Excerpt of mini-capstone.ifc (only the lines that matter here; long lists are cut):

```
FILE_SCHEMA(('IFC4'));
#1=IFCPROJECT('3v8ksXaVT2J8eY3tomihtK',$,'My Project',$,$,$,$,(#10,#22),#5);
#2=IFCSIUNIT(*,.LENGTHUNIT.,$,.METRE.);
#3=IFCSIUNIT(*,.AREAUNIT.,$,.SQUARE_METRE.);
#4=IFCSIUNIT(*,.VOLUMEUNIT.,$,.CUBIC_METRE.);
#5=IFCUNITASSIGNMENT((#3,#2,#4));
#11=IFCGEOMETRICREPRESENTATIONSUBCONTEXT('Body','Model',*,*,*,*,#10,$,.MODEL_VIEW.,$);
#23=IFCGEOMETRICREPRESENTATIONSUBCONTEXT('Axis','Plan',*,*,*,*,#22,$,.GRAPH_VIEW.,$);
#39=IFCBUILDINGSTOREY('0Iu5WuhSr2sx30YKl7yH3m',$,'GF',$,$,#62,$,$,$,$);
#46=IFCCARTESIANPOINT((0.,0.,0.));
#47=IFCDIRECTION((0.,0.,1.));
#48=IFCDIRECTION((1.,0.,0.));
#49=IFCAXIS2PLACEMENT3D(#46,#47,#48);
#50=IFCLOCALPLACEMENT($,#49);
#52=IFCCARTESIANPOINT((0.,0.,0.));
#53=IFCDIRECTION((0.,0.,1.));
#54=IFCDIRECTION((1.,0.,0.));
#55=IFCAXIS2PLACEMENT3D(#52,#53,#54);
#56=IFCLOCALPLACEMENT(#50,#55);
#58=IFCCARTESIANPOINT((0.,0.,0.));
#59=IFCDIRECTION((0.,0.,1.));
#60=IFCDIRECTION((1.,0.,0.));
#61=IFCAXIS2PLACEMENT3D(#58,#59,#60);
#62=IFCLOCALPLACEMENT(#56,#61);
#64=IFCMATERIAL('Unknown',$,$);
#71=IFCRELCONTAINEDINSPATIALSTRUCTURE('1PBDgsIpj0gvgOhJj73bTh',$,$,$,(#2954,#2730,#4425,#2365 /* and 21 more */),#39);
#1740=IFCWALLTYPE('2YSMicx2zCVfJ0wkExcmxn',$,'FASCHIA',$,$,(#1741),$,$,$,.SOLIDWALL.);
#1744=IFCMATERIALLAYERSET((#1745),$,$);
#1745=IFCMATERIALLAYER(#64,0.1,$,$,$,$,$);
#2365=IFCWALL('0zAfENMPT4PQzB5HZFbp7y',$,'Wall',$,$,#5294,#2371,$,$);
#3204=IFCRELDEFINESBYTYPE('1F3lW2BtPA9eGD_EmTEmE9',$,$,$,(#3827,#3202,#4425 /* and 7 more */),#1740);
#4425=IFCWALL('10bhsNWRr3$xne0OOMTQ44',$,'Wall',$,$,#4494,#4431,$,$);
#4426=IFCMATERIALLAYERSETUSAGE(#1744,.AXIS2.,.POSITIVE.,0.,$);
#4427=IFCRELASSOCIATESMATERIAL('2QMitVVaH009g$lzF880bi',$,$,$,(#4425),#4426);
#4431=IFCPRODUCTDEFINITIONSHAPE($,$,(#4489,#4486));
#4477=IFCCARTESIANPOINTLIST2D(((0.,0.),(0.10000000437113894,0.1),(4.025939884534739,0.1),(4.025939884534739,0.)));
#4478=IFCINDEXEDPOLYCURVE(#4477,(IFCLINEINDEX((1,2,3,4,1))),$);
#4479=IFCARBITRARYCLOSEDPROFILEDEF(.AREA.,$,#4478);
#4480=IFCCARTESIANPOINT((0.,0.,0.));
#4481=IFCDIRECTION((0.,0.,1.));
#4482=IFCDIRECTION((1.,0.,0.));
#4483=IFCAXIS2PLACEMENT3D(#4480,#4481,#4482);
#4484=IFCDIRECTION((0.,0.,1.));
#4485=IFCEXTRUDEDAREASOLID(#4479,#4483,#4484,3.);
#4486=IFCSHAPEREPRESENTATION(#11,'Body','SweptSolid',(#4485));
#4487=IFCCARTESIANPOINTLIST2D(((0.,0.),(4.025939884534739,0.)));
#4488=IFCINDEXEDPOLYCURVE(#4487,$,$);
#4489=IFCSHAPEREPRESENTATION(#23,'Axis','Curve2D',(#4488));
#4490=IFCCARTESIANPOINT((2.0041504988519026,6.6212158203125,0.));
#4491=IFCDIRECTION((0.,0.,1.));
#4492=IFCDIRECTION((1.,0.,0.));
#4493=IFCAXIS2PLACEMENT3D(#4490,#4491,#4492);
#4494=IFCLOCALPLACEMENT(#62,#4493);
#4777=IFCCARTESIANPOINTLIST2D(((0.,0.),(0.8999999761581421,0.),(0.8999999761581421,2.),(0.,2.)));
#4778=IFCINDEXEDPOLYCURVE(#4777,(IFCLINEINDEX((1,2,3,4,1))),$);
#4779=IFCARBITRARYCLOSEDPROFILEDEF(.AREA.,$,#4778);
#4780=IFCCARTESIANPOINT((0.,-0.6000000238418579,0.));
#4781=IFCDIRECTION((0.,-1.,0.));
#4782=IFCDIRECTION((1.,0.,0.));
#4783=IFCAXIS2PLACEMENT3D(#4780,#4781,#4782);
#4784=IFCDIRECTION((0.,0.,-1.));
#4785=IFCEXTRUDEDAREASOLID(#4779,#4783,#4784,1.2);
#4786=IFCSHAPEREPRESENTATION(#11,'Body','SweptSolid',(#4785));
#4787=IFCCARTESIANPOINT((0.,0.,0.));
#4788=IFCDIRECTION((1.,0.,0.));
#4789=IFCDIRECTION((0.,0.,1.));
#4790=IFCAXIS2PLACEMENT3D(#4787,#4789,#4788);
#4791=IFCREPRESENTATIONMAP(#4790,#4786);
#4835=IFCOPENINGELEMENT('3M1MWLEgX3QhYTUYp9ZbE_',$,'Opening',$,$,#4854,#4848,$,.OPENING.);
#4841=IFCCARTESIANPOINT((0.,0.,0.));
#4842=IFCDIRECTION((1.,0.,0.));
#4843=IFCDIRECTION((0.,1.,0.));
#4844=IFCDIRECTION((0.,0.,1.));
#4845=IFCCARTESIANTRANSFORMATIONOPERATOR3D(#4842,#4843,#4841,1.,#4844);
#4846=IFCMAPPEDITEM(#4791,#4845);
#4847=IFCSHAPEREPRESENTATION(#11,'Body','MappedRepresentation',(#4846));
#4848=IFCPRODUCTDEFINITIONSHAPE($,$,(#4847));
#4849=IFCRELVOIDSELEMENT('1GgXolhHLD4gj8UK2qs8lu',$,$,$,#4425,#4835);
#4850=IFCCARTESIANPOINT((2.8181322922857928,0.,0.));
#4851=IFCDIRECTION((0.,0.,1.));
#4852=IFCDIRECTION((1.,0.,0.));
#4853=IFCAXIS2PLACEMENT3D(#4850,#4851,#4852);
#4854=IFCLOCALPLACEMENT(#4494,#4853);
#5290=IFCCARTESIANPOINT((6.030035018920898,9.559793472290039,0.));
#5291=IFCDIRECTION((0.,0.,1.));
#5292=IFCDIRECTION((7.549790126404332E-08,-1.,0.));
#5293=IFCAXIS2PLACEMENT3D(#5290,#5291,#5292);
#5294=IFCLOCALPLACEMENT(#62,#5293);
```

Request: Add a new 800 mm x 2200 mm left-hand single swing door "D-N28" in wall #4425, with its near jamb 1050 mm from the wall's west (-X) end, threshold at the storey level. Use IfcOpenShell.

```python
import numpy as np
import ifcopenshell
import ifcopenshell.api.feature
import ifcopenshell.api.geometry
import ifcopenshell.api.root
import ifcopenshell.api.spatial
import ifcopenshell.geom
import ifcopenshell.util.element
import ifcopenshell.util.placement
import ifcopenshell.util.representation
import ifcopenshell.util.shape
import ifcopenshell.util.unit

model = ifcopenshell.open("mini-capstone.ifc")
unit_scale = ifcopenshell.util.unit.calculate_unit_scale(model)
settings = ifcopenshell.geom.settings()


def volume(element):
    """Net volume in cubic metres, openings subtracted."""
    shape = ifcopenshell.geom.create_shape(settings, element)
    return ifcopenshell.util.shape.get_volume(shape.geometry)


wall = model.by_id(4425)
storey = ifcopenshell.util.element.get_container(wall, ifc_class="IfcBuildingStorey")
context = ifcopenshell.util.representation.get_context(model, "Model", "Body", "MODEL_VIEW")
before = volume(wall)

width, height, from_end, sill = 0.8, 2.2, 1.05, 0.0  # metres

# The wall runs along its own X axis, and the end named is its -X end.
wall_shape = ifcopenshell.geom.create_shape(settings, wall)
x, y, z = ifcopenshell.util.shape.get_vertices(wall_shape.geometry).T
start = x.min() + from_end
face, thickness = float(y.min()), float(y.max() - y.min())
wall_matrix = ifcopenshell.util.placement.get_local_placement(wall.ObjectPlacement)
level = ifcopenshell.util.placement.get_local_placement(storey.ObjectPlacement)[2, 3]


def in_wall(x, y):
    """Placement at x, y metres in the wall's axes, at sill height."""
    matrix = wall_matrix.copy()
    matrix[:, 3] = wall_matrix @ np.array([x / unit_scale, y / unit_scale, 0.0, 1.0])
    matrix[2, 3] = level + sill / unit_scale
    return matrix


# Opening: a box that overshoots both wall faces by 50 mm.
opening = ifcopenshell.api.root.create_entity(model, ifc_class="IfcOpeningElement", predefined_type="OPENING")
box = ifcopenshell.api.geometry.add_wall_representation(
    model, context=context, length=width, height=height, thickness=thickness + 0.1
)
ifcopenshell.api.geometry.assign_representation(model, product=opening, representation=box)
ifcopenshell.api.geometry.edit_object_placement(model, product=opening, matrix=in_wall(start, face - 0.05), is_si=False)
ifcopenshell.api.feature.add_feature(model, feature=opening, element=wall)

door = ifcopenshell.api.root.create_entity(model, ifc_class="IfcDoor", name="D-N28", predefined_type="DOOR")
door.OverallWidth, door.OverallHeight = width / unit_scale, height / unit_scale
door.OperationType = "SINGLE_SWING_LEFT"
body = ifcopenshell.api.geometry.add_door_representation(
    model,
    context=context,
    overall_width=door.OverallWidth,
    overall_height=door.OverallHeight,
    operation_type="SINGLE_SWING_LEFT",
    lining_properties={"LiningDepth": thickness / unit_scale, "ThresholdDepth": thickness / unit_scale},
)
ifcopenshell.api.geometry.assign_representation(model, product=door, representation=body)
ifcopenshell.api.spatial.assign_container(model, products=[door], relating_structure=storey)
ifcopenshell.api.feature.add_filling(model, opening=opening, element=door)

# The lining spans the wall, so the door starts at the wall face.
ifcopenshell.api.geometry.edit_object_placement(model, product=door, matrix=in_wall(start, face), is_si=False)

after = volume(wall)

print(f"wall volume {before:.3f} -> {after:.3f} m3")

model.write("mini-capstone-out.ifc")
```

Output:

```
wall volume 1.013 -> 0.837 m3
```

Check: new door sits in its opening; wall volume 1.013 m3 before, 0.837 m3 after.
